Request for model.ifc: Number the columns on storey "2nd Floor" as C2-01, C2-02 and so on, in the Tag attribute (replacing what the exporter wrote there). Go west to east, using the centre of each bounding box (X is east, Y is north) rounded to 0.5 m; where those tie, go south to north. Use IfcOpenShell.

First a look at what the model holds.

```python
import ifcopenshell
import ifcopenshell.util.element
import ifcopenshell.util.placement

model = ifcopenshell.open("model.ifc")
print(model.schema)
storey = next(s for s in model.by_type("IfcBuildingStorey") if s.Name == "2nd Floor")
columns = [e for e in ifcopenshell.util.element.get_decomposition(storey) if e.is_a("IfcColumn")]
for e in sorted(columns, key=lambda e: e.id()):
    origin = ifcopenshell.util.placement.get_local_placement(e.ObjectPlacement)[:3, 3]
    print(e.id(), e.Tag, e.Name, origin.round(2) + 0.0, sep=" | ")
```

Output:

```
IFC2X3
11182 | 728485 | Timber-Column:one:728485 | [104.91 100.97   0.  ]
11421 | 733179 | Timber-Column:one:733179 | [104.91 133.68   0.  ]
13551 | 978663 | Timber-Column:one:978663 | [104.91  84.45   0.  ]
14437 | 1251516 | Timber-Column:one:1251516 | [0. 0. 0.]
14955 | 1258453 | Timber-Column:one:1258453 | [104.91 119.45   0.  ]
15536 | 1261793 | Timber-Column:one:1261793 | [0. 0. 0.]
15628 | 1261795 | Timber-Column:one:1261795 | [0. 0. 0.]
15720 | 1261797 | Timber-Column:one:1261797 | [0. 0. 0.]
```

```python
import ifcopenshell
import ifcopenshell.geom
import ifcopenshell.util.element
import ifcopenshell.util.shape

model = ifcopenshell.open("model.ifc")
settings = ifcopenshell.geom.settings()
settings.set("use-world-coords", True)


def centre(element):
    shape = ifcopenshell.geom.create_shape(settings, element)
    return ifcopenshell.util.shape.get_bbox_centroid(shape.geometry)


storey = next(s for s in model.by_type("IfcBuildingStorey") if s.Name == "2nd Floor")
columns = [e for e in ifcopenshell.util.element.get_decomposition(storey) if e.is_a("IfcColumn")]

# Insertion points can sit at a corner or the storey origin, so sort by the geometry (in metres).
centres = {e: centre(e) for e in columns}
columns.sort(key=lambda e: (round(centres[e][0] / 0.5), centres[e][1]))

for i, e in enumerate(columns, start=1):
    number = f"C2-{i:02d}"
    e.Tag = number
    print(e.id(), number)

model.write("model_updated.ifc")
```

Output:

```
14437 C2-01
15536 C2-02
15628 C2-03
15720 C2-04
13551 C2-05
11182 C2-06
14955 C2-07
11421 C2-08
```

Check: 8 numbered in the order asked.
